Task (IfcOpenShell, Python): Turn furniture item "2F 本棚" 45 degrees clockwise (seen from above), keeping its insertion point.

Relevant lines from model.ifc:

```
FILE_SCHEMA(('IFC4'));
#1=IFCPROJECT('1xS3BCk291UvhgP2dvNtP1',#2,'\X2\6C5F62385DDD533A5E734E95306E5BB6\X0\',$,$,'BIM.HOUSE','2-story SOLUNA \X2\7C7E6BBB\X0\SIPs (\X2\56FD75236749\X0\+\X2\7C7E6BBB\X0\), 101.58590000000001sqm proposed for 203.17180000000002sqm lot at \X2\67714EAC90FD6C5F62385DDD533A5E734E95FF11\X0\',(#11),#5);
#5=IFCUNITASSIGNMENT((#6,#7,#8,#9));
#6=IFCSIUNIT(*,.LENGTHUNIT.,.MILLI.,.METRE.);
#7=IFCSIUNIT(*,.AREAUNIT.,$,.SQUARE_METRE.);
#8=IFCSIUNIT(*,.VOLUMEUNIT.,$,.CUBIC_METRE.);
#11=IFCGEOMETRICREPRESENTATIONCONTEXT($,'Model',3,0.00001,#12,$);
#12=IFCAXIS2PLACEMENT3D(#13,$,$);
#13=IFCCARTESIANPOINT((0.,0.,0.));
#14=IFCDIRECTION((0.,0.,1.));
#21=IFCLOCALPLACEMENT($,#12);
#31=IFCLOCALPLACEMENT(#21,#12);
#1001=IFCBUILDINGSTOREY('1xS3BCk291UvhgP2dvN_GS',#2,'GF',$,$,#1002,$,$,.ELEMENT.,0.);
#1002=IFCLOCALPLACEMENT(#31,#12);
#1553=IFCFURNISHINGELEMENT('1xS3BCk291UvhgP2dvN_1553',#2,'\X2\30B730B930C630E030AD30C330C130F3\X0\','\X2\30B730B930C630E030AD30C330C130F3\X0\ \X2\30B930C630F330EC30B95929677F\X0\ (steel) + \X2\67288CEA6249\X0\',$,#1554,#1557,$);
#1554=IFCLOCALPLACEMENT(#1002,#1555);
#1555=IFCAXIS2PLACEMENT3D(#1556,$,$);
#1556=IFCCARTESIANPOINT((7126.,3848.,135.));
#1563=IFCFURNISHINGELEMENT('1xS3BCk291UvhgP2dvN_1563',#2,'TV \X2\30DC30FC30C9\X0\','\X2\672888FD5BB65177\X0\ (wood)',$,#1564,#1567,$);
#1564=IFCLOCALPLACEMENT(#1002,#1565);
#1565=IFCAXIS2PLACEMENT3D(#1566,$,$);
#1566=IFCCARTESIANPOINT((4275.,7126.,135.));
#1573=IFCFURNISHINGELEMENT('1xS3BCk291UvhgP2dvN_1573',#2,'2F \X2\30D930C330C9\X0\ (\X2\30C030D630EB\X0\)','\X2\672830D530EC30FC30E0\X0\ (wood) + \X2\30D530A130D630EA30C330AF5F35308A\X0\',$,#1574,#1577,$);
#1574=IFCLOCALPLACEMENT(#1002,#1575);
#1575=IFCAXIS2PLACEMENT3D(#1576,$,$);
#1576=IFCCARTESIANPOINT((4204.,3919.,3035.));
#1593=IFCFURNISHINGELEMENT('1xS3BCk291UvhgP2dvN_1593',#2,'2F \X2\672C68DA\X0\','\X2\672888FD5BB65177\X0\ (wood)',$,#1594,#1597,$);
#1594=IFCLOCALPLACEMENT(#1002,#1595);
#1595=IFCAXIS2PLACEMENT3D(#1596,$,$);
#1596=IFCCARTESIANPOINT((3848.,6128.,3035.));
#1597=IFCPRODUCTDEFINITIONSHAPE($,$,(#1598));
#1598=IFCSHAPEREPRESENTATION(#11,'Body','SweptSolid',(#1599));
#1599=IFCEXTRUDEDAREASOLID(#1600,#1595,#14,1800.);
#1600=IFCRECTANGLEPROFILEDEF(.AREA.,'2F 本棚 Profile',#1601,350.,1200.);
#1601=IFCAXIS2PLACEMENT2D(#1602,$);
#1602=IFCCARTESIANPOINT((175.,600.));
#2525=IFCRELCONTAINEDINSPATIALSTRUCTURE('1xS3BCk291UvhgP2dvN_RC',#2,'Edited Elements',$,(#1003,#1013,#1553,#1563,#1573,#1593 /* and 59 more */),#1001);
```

```python
import ifcopenshell
import ifcopenshell.api.geometry
import ifcopenshell.util.placement

model = ifcopenshell.open("model.ifc")

item = model.by_guid("1xS3BCk291UvhgP2dvN_1593")
matrix = ifcopenshell.util.placement.get_local_placement(item.ObjectPlacement)
matrix = matrix @ ifcopenshell.util.placement.rotation(-45, "Z")
ifcopenshell.api.geometry.edit_object_placement(model, product=item, matrix=matrix, is_si=False)

print(ifcopenshell.util.placement.get_local_placement(item.ObjectPlacement).round(3) + 0.0)

model.write("model-out.ifc")
```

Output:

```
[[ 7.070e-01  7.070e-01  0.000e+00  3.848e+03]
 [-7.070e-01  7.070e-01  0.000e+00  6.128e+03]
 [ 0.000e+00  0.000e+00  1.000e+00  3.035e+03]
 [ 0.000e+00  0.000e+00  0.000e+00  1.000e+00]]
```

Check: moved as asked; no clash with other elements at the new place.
